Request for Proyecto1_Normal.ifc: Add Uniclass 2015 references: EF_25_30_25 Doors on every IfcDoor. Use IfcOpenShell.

First a look at what the model holds.

```python
import ifcopenshell

model = ifcopenshell.open("Proyecto1_Normal.ifc")
print(model.schema)
print("classifications:", [c.Name for c in model.by_type("IfcClassification")])
for ifc_class in ("IfcDoor", "IfcRoof", "IfcStair", "IfcWall", "IfcWindow"):
    print(ifc_class, len(model.by_type(ifc_class)))
```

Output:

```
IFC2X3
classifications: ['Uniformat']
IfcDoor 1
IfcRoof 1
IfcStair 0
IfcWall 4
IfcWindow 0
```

```python
import ifcopenshell
import ifcopenshell.api.classification

model = ifcopenshell.open("Proyecto1_Normal.ifc")

# IFC2X3 requires Source and Edition and has no link from the project to the system.
system = model.create_entity("IfcClassification", Source="NBS", Edition="2015", Name="Uniclass 2015")

codes = {
    "IfcDoor": ("EF_25_30_25", "Doors"),
}
for ifc_class, (code, name) in codes.items():
    products = model.by_type(ifc_class)
    ifcopenshell.api.classification.add_reference(
        model, products=products, classification=system, identification=code, name=name
    )
    print(code, len(products))

model.write("Proyecto1_Normal_updated.ifc")
```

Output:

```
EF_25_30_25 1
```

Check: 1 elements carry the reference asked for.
